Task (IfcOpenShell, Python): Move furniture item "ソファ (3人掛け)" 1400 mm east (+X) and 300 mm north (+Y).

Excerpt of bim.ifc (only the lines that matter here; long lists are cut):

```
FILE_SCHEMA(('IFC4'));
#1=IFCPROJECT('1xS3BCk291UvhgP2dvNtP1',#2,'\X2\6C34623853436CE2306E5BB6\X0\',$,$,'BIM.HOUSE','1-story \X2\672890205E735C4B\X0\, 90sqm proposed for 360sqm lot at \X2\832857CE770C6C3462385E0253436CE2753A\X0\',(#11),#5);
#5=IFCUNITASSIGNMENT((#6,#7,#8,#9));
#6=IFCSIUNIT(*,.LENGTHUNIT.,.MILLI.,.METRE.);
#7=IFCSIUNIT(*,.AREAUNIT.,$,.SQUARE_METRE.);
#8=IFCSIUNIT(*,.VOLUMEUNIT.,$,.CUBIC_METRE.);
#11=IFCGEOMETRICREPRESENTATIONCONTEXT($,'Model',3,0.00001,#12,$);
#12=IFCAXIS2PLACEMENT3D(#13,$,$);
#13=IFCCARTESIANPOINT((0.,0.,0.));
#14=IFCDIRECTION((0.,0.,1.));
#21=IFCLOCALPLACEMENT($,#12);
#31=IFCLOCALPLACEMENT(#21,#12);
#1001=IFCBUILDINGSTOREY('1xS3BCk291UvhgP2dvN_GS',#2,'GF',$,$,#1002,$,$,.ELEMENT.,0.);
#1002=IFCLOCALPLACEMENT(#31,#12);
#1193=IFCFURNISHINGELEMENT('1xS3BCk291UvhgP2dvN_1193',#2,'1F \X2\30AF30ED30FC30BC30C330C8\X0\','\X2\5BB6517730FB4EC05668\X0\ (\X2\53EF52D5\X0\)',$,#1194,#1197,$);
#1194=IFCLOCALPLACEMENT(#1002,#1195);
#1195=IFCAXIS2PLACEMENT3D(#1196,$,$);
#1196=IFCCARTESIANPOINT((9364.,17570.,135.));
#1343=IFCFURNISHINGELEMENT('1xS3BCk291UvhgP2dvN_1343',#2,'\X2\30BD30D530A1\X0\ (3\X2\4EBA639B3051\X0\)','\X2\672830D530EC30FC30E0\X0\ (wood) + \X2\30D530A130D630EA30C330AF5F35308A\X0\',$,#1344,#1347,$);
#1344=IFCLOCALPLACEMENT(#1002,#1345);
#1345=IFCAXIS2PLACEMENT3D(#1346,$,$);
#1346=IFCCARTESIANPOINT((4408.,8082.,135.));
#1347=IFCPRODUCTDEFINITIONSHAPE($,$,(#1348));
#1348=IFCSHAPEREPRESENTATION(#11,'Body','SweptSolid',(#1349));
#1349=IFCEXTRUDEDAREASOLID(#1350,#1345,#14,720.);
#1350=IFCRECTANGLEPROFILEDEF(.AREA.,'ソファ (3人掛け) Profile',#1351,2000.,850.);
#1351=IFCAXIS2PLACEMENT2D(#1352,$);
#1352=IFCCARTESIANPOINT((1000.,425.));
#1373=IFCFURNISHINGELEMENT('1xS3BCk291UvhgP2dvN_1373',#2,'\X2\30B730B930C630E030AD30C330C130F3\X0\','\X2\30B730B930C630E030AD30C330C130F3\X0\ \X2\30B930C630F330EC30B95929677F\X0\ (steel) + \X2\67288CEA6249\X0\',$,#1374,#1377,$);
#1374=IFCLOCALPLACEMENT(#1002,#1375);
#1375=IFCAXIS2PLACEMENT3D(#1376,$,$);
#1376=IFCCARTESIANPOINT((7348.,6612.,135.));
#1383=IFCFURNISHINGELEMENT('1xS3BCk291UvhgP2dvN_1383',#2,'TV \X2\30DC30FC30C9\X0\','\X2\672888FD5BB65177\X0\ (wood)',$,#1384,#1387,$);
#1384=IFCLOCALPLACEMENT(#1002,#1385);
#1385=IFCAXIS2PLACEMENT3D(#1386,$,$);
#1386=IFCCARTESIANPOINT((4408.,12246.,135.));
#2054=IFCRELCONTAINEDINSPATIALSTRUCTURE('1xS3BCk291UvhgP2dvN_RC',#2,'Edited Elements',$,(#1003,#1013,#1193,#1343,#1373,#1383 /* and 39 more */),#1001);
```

```python
import ifcopenshell
import ifcopenshell.api.geometry
import ifcopenshell.util.placement

model = ifcopenshell.open("bim.ifc")

item = model.by_guid("1xS3BCk291UvhgP2dvN_1343")
matrix = ifcopenshell.util.placement.get_local_placement(item.ObjectPlacement)
matrix[0, 3] += 1400.0
matrix[1, 3] += 300.0
ifcopenshell.api.geometry.edit_object_placement(model, product=item, matrix=matrix, is_si=False)

print(ifcopenshell.util.placement.get_local_placement(item.ObjectPlacement).round(3) + 0.0)

model.write("bim_edited.ifc")
```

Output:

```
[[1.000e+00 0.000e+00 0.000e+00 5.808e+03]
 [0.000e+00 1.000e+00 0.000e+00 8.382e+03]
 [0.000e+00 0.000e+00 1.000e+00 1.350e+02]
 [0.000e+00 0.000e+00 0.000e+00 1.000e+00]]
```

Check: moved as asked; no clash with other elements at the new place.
